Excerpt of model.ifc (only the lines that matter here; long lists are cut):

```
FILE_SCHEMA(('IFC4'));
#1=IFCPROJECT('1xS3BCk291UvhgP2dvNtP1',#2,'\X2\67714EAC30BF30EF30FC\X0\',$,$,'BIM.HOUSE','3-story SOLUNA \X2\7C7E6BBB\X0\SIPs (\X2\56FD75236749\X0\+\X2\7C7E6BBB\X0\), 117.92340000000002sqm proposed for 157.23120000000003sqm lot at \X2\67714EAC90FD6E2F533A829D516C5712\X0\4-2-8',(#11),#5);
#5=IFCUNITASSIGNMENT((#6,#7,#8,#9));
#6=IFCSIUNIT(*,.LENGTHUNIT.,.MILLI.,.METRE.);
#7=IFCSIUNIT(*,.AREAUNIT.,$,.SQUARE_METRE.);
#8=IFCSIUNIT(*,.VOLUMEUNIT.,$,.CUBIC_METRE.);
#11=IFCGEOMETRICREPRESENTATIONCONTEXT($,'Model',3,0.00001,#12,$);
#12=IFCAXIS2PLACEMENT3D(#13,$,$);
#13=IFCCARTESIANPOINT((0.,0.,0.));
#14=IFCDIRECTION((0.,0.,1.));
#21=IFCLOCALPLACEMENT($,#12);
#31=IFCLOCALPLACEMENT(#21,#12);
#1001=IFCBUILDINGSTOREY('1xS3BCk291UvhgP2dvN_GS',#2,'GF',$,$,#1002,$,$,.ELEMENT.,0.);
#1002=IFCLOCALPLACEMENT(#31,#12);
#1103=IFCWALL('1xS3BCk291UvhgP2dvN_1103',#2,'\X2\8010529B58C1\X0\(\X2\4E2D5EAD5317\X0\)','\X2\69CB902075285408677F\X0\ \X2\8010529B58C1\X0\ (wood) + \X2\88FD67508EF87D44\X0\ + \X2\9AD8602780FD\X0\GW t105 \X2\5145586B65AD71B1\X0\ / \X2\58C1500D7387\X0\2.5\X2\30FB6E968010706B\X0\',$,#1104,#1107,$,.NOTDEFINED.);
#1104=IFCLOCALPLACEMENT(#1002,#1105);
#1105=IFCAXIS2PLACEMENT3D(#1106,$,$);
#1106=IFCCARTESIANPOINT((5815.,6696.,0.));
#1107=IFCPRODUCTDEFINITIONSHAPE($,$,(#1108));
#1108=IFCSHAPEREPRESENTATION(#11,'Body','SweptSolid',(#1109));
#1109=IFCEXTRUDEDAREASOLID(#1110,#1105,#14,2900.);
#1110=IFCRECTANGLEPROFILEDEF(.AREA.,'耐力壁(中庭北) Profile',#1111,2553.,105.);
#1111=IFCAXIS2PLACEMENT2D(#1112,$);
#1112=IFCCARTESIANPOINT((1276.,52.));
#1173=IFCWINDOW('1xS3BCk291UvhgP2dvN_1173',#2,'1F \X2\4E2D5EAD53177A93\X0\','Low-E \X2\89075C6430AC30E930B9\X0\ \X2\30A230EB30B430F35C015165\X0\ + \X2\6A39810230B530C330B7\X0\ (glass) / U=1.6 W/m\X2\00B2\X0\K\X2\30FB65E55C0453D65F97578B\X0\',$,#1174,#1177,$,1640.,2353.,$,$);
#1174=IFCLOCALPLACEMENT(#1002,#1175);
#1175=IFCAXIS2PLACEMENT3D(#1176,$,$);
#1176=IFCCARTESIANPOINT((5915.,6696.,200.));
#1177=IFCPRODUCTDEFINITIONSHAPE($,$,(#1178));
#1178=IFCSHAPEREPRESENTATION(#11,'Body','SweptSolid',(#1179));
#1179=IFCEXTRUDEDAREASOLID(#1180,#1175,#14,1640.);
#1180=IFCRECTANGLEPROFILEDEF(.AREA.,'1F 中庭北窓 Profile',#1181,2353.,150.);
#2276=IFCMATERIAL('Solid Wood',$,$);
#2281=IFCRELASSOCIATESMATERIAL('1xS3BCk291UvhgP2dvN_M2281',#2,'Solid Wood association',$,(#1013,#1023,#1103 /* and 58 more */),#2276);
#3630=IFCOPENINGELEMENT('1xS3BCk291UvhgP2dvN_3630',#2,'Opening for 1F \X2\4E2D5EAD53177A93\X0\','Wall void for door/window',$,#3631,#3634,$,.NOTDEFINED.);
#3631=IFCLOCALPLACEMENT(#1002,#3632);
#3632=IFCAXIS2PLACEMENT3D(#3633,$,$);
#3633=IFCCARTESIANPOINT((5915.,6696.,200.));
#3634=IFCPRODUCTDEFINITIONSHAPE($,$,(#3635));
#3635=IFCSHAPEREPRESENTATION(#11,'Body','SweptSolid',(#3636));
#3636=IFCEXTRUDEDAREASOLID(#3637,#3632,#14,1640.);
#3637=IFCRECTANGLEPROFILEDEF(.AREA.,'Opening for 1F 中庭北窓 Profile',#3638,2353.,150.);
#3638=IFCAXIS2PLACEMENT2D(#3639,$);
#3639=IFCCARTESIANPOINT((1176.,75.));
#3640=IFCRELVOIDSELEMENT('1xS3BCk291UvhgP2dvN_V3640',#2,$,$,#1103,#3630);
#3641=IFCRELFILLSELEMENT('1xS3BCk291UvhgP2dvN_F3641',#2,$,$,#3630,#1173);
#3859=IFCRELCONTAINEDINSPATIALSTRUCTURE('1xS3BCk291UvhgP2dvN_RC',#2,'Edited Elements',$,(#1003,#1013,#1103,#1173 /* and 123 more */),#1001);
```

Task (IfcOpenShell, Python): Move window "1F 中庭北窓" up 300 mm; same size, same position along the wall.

```python
import numpy as np
import ifcopenshell
import ifcopenshell.api.geometry
import ifcopenshell.util.placement
import ifcopenshell.util.unit

model = ifcopenshell.open("model.ifc")
unit_scale = ifcopenshell.util.unit.calculate_unit_scale(model)

window = model.by_guid("1xS3BCk291UvhgP2dvN_1173")
opening = window.FillsVoids[0].RelatingOpeningElement
dz = 300.0

shift = np.array([0.0, 0.0, dz])
# The window is not placed relative to its opening, so move both.
for product in (opening, window):
    matrix = ifcopenshell.util.placement.get_local_placement(product.ObjectPlacement)
    matrix[:3, 3] += shift
    ifcopenshell.api.geometry.edit_object_placement(model, product=product, matrix=matrix, is_si=False)

print(f"moved by {dz * unit_scale:+.3f} m")

model.write("model_edited.ifc")
```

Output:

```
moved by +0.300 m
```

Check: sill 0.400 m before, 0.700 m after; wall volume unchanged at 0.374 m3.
